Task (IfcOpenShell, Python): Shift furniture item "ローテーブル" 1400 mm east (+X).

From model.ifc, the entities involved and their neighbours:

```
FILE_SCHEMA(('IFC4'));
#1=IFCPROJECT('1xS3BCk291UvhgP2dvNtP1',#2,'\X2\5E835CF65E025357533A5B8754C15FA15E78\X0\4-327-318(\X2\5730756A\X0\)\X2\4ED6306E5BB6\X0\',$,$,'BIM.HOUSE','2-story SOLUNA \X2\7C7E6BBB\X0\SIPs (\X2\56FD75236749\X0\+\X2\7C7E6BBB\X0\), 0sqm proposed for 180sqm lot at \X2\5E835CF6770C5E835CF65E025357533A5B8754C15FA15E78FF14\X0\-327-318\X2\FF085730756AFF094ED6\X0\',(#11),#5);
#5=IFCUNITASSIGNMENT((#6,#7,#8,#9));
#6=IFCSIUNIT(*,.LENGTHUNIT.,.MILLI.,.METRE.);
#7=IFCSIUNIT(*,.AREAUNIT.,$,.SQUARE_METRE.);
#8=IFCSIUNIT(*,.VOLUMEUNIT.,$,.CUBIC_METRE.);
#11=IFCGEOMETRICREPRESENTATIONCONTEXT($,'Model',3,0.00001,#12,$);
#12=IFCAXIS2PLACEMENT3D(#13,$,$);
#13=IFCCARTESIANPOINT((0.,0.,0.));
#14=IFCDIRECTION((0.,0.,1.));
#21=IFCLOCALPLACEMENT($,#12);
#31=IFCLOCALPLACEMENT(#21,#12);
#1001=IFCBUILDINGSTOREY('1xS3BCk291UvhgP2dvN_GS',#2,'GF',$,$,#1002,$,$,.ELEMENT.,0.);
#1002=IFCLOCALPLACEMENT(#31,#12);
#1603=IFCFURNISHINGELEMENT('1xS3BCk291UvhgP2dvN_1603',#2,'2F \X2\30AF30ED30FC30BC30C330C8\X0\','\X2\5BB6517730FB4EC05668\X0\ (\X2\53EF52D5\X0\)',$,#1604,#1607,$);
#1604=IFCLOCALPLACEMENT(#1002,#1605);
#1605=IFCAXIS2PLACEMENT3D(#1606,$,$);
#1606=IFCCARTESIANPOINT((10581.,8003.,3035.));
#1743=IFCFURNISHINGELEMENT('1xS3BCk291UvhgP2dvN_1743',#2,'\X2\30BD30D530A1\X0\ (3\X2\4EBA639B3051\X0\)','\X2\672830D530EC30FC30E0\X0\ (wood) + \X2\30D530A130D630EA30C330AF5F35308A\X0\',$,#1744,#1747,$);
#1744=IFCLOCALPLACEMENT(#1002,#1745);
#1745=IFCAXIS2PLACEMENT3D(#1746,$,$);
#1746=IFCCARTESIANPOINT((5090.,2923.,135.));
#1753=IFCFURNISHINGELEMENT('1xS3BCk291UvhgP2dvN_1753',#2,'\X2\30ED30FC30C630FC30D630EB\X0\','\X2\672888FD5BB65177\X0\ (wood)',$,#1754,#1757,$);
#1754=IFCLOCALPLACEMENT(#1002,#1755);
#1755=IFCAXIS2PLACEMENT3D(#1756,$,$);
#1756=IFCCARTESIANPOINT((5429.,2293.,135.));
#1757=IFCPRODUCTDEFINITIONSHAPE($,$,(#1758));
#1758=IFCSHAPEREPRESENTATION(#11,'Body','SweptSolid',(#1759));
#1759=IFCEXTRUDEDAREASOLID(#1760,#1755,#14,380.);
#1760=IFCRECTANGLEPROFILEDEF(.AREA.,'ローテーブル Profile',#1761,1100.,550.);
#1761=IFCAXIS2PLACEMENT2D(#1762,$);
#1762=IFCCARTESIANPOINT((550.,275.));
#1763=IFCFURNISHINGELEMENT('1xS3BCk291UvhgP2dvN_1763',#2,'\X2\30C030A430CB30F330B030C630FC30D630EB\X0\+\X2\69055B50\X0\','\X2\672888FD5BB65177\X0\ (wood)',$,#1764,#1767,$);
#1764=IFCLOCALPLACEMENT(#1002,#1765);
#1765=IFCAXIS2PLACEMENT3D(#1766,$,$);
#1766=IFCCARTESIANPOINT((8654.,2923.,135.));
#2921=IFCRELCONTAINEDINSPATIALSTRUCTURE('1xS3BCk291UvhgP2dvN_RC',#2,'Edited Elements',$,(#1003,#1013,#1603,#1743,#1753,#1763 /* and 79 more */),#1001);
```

```python
import ifcopenshell
import ifcopenshell.api.geometry
import ifcopenshell.util.placement

model = ifcopenshell.open("model.ifc")

item = model.by_guid("1xS3BCk291UvhgP2dvN_1753")
matrix = ifcopenshell.util.placement.get_local_placement(item.ObjectPlacement)
matrix[0, 3] += 1400.0
ifcopenshell.api.geometry.edit_object_placement(model, product=item, matrix=matrix, is_si=False)

print(ifcopenshell.util.placement.get_local_placement(item.ObjectPlacement).round(3) + 0.0)

model.write("model-out.ifc")
```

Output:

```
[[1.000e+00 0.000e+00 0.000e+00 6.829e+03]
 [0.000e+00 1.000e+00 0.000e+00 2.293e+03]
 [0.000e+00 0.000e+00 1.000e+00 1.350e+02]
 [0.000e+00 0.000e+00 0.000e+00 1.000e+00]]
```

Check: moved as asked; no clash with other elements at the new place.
